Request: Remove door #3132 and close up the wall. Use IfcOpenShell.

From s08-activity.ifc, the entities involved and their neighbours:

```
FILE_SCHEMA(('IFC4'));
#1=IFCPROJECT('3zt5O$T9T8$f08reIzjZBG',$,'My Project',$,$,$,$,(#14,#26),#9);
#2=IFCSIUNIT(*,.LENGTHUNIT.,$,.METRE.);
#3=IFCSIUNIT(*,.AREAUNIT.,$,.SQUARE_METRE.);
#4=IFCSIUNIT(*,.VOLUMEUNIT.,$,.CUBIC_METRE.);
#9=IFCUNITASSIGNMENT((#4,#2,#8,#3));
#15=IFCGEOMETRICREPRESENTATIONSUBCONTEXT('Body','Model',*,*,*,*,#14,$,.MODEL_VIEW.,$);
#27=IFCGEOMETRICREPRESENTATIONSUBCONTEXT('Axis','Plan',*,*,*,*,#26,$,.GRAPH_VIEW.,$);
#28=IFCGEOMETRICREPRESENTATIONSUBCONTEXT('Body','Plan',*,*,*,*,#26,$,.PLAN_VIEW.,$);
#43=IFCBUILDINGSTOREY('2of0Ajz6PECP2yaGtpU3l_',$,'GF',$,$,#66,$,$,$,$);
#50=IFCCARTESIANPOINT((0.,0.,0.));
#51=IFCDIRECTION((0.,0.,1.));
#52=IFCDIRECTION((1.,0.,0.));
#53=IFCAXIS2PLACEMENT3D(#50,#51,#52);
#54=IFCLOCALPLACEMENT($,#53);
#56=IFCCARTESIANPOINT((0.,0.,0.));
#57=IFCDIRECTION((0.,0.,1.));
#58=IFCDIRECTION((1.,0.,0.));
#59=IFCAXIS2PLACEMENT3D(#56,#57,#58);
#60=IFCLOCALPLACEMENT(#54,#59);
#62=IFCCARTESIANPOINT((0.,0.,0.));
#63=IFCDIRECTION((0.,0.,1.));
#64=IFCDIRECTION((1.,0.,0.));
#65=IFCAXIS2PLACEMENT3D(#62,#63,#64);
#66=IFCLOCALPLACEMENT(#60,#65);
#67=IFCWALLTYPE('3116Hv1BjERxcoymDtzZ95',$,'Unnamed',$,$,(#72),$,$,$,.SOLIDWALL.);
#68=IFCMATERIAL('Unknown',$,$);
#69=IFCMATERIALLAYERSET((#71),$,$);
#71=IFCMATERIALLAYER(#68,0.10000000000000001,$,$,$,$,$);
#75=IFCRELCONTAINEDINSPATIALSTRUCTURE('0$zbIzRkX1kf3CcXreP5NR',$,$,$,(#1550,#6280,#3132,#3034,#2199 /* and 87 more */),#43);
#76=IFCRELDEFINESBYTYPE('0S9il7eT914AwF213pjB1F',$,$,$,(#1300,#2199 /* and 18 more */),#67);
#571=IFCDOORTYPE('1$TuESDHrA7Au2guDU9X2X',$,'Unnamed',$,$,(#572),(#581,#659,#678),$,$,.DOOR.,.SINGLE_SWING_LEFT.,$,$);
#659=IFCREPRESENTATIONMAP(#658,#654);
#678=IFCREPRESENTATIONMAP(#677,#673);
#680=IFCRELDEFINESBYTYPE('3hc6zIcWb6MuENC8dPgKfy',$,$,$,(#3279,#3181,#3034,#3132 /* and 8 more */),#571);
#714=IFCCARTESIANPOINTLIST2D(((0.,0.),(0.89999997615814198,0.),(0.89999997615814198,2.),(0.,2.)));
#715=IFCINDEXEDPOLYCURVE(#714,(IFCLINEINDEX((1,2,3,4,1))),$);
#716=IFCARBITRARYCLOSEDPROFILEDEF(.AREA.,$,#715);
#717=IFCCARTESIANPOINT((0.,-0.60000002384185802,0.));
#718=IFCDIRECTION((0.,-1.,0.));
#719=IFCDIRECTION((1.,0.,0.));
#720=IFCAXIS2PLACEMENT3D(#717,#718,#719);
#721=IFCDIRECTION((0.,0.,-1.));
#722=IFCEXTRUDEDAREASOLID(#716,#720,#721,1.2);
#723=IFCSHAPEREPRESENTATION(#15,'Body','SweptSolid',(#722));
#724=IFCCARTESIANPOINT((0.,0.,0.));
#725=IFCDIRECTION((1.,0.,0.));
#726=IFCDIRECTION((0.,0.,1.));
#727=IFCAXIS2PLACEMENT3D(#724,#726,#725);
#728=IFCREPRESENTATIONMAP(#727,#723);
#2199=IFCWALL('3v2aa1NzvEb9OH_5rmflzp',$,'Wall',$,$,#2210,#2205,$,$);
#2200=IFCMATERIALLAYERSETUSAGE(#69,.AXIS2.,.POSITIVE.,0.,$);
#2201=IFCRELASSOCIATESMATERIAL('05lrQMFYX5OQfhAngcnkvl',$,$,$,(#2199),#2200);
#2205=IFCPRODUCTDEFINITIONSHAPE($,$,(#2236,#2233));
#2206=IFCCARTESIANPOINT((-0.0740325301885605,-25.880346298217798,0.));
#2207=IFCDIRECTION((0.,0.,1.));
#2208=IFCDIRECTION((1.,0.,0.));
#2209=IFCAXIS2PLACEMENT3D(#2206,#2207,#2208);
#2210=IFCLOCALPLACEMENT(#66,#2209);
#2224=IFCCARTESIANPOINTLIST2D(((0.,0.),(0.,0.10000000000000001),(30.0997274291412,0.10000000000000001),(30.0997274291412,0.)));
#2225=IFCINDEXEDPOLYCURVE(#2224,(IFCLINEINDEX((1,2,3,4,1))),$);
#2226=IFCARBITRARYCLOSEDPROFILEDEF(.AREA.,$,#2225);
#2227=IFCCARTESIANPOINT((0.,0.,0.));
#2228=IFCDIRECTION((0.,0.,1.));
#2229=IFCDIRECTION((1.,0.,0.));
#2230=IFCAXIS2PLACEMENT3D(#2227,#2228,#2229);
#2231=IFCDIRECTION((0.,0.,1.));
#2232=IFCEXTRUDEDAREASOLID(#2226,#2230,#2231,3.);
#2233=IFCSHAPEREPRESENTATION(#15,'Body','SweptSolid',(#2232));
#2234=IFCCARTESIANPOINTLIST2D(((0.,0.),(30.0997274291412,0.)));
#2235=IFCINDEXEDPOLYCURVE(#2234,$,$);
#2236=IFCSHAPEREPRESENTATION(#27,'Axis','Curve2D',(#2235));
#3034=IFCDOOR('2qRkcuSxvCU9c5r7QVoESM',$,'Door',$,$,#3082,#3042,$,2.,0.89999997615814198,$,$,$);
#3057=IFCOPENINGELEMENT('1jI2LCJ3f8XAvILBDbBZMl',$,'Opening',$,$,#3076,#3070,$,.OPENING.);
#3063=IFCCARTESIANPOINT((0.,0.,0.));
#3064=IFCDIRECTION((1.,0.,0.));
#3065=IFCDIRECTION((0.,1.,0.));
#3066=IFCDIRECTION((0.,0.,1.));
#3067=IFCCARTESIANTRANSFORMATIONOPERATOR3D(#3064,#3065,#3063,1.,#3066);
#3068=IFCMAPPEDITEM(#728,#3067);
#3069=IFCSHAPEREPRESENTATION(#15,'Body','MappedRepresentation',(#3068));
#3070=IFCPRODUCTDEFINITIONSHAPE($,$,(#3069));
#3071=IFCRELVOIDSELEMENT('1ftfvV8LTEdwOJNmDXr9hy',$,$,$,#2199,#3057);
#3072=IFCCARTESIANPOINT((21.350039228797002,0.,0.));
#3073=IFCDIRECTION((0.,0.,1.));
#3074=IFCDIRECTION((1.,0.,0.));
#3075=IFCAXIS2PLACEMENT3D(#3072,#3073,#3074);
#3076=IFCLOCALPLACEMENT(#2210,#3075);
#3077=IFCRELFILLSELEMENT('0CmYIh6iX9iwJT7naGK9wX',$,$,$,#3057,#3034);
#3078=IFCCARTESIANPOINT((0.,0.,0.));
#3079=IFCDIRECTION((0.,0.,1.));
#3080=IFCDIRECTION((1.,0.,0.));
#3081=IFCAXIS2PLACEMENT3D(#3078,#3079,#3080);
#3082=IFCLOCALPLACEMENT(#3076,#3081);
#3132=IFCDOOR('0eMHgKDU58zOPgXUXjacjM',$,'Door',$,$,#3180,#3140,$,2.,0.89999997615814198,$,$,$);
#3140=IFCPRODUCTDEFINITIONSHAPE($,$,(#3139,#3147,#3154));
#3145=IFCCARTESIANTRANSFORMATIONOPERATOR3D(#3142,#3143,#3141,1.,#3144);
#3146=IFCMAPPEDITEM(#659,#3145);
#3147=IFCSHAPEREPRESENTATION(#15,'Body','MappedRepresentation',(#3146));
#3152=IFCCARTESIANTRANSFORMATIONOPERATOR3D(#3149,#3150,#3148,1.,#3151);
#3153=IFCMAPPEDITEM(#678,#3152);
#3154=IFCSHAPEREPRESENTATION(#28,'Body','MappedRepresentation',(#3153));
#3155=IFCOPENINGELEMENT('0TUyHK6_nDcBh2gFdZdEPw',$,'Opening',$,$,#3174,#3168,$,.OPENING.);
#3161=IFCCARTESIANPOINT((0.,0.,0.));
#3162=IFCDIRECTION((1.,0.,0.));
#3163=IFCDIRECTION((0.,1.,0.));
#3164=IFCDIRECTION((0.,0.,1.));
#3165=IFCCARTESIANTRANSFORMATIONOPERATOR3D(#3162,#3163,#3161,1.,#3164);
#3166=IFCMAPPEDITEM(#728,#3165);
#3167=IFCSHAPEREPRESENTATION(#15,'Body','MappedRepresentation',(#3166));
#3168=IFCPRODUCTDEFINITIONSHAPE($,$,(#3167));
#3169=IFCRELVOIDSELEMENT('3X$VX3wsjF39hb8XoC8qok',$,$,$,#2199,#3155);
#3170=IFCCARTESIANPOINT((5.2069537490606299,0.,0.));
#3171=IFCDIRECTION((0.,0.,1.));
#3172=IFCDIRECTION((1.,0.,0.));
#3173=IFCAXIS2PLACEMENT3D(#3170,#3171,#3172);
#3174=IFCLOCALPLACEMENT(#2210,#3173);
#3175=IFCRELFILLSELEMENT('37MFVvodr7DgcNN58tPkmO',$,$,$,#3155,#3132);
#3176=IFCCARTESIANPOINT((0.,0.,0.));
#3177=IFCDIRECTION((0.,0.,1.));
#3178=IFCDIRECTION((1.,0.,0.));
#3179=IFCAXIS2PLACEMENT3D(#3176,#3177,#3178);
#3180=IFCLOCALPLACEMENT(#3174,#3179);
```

```python
import ifcopenshell
import ifcopenshell.api.feature
import ifcopenshell.api.root
import ifcopenshell.geom
import ifcopenshell.util.shape

model = ifcopenshell.open("s08-activity.ifc")
settings = ifcopenshell.geom.settings()


def volume(element):
    """Net volume in cubic metres, openings subtracted."""
    shape = ifcopenshell.geom.create_shape(settings, element)
    return ifcopenshell.util.shape.get_volume(shape.geometry)


door = model.by_guid("0eMHgKDU58zOPgXUXjacjM")
opening = door.FillsVoids[0].RelatingOpeningElement
wall = opening.VoidsElements[0].RelatingBuildingElement
before = volume(wall)

ifcopenshell.api.root.remove_product(model, product=door)
ifcopenshell.api.feature.remove_feature(model, feature=opening)

after = volume(wall)

print(f"wall volume {before:.3f} -> {after:.3f} m3")

model.write("s08-activity_v2.ifc")
```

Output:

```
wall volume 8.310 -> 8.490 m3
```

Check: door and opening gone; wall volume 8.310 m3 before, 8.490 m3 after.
